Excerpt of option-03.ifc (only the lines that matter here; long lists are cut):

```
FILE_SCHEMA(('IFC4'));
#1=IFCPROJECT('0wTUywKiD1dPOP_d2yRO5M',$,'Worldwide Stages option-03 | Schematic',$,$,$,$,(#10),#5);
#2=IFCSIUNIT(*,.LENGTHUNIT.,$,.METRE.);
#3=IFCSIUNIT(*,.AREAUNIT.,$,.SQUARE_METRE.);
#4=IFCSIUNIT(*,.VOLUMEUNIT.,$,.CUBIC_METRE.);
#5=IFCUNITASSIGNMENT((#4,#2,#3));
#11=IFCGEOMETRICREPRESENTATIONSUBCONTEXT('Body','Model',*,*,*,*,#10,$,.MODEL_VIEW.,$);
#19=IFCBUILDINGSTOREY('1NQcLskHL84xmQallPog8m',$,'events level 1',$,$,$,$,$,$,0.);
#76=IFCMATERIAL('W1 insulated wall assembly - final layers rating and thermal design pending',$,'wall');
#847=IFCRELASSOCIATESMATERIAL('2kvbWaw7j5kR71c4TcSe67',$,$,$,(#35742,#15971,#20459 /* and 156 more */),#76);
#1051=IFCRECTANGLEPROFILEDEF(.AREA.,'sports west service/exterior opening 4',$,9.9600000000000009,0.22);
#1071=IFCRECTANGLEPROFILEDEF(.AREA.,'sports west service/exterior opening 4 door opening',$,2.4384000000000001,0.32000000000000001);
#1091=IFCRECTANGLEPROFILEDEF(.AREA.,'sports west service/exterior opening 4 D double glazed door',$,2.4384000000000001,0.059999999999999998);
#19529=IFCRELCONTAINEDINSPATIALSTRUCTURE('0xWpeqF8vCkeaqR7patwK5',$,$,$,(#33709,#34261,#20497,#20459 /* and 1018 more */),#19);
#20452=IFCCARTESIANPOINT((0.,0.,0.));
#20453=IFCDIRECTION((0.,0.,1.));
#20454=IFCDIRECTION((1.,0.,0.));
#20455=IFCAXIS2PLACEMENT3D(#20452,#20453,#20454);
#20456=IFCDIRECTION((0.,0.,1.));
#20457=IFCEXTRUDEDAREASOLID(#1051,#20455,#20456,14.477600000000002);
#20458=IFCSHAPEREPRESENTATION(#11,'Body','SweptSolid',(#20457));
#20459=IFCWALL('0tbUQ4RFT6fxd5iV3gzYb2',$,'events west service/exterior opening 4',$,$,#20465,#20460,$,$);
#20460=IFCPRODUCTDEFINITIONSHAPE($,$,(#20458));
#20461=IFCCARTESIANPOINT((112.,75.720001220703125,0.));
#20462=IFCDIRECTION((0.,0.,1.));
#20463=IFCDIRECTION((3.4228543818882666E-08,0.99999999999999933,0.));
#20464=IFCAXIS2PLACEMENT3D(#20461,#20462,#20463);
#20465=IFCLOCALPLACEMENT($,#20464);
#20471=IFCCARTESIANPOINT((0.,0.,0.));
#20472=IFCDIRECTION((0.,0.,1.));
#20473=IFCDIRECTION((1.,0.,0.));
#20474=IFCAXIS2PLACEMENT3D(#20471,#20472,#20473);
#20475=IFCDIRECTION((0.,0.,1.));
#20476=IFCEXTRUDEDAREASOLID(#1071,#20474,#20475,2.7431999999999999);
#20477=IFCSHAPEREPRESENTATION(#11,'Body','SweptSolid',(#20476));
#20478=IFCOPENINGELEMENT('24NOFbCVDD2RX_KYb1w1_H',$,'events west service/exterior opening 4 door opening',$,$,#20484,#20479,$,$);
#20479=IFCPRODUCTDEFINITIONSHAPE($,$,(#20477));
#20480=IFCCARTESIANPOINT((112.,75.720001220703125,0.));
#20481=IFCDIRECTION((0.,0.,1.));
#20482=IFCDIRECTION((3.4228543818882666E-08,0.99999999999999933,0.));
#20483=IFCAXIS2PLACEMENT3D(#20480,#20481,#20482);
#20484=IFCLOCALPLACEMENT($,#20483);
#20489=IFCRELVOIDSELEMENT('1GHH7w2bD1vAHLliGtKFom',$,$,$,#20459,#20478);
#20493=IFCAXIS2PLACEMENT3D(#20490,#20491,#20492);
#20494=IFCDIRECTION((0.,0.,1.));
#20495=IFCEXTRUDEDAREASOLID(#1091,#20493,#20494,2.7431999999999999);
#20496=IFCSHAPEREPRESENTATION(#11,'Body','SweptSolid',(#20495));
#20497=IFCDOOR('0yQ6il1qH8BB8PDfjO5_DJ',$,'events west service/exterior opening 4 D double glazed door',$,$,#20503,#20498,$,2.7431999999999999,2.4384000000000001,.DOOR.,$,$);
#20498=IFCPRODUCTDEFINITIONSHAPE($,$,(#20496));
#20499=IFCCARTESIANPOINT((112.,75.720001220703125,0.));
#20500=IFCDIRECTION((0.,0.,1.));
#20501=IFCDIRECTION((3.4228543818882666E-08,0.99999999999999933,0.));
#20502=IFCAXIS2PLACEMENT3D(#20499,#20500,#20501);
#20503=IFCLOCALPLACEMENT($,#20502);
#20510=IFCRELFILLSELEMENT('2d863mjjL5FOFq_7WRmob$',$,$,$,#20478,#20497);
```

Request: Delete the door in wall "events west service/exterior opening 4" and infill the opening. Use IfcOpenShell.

```python
import ifcopenshell
import ifcopenshell.api.feature
import ifcopenshell.api.root
import ifcopenshell.geom
import ifcopenshell.util.shape

model = ifcopenshell.open("option-03.ifc")
settings = ifcopenshell.geom.settings()


def volume(element):
    """Net volume in cubic metres, openings subtracted."""
    shape = ifcopenshell.geom.create_shape(settings, element)
    return ifcopenshell.util.shape.get_volume(shape.geometry)


door = model.by_guid("0yQ6il1qH8BB8PDfjO5_DJ")
opening = door.FillsVoids[0].RelatingOpeningElement
wall = opening.VoidsElements[0].RelatingBuildingElement
before = volume(wall)

ifcopenshell.api.root.remove_product(model, product=door)
ifcopenshell.api.feature.remove_feature(model, feature=opening)

after = volume(wall)

print(f"wall volume {before:.3f} -> {after:.3f} m3")

model.write("option-03_edited.ifc")
```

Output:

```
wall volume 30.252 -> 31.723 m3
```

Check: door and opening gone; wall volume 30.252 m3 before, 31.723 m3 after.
